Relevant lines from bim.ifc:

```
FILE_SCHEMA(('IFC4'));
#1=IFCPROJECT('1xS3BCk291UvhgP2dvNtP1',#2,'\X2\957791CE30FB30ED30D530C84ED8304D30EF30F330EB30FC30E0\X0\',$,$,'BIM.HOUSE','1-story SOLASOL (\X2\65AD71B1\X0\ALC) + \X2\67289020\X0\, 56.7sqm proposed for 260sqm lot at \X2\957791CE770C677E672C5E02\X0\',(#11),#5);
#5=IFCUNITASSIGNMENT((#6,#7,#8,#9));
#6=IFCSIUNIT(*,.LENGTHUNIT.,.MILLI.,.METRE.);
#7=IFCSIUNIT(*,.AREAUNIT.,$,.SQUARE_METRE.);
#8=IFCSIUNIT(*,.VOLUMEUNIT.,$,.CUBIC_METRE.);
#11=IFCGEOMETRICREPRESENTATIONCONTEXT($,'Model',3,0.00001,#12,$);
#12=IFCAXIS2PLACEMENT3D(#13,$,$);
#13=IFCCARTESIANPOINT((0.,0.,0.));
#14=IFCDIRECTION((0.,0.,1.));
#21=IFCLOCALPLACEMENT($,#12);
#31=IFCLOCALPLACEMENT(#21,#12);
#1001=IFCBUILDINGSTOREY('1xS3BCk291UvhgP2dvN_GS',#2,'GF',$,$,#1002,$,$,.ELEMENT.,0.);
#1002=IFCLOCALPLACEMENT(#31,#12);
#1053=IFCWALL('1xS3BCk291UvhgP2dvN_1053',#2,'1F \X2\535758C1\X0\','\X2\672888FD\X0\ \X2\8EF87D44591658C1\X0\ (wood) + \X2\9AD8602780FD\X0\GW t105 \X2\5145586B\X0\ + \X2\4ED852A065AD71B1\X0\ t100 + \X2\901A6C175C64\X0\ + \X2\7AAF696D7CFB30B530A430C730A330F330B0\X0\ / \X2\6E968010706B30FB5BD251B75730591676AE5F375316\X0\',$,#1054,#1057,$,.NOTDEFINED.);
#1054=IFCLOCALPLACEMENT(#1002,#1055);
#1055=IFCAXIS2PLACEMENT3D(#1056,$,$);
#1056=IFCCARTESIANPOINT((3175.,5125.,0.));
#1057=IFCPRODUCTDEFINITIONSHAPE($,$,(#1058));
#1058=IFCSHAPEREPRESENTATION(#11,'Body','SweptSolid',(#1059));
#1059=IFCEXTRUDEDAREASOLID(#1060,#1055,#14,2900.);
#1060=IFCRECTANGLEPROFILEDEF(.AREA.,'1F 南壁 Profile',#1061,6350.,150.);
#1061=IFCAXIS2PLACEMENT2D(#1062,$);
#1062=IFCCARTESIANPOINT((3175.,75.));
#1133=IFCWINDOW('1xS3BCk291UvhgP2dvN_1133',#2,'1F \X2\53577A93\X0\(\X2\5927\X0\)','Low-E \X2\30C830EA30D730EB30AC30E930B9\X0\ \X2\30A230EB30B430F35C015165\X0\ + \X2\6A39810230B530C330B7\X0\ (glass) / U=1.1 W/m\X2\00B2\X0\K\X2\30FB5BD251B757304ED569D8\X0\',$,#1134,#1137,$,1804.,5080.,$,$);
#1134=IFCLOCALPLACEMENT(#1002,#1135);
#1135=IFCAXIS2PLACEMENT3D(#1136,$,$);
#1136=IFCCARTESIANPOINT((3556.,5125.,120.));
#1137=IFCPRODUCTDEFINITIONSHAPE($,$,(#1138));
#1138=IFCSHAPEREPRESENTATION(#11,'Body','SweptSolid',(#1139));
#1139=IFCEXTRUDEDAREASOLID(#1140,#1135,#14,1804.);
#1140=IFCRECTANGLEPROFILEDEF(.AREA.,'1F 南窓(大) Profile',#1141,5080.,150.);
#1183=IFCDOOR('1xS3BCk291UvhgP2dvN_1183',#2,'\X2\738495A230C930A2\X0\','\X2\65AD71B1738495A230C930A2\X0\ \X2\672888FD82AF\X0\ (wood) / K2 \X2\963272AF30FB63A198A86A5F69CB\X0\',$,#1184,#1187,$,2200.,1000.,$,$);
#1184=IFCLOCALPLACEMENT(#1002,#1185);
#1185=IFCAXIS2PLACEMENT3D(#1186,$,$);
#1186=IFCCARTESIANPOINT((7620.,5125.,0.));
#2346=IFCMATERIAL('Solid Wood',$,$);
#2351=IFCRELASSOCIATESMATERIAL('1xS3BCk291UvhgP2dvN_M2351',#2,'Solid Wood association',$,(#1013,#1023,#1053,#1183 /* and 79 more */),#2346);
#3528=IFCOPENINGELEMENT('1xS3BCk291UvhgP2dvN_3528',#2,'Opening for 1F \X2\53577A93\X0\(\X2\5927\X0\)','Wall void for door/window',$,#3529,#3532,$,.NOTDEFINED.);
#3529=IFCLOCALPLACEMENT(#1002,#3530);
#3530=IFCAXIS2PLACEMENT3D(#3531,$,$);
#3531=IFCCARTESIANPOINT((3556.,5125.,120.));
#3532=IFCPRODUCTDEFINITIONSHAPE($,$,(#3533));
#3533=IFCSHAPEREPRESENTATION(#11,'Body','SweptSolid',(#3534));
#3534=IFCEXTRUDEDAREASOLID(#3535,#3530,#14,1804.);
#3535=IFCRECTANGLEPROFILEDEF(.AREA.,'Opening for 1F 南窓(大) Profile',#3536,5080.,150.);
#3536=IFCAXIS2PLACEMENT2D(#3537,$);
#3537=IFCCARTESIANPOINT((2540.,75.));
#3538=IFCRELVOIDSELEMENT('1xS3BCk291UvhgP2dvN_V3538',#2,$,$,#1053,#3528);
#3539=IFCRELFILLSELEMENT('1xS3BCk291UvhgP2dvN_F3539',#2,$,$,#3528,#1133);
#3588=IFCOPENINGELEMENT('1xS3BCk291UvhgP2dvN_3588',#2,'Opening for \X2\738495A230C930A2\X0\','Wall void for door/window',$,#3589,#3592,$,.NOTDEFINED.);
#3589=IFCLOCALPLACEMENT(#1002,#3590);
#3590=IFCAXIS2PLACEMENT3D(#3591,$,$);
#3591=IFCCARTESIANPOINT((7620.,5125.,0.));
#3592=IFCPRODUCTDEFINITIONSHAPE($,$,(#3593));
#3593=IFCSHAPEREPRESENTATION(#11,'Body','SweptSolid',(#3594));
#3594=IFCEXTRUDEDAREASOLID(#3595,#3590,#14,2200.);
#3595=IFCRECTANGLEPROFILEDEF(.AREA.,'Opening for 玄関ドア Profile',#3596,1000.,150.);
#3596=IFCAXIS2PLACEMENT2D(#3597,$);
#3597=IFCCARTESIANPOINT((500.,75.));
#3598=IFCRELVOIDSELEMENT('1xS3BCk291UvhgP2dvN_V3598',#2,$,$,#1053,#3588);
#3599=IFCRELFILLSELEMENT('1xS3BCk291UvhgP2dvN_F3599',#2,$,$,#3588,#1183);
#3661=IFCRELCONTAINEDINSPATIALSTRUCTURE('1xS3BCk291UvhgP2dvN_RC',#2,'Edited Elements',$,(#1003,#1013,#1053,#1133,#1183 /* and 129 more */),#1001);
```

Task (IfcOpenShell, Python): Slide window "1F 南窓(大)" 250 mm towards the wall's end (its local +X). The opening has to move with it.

```python
import ifcopenshell
import ifcopenshell.api.geometry
import ifcopenshell.util.placement

model = ifcopenshell.open("bim.ifc")

window = model.by_id(1133)
opening = window.FillsVoids[0].RelatingOpeningElement
wall = opening.VoidsElements[0].RelatingBuildingElement

wall_matrix = ifcopenshell.util.placement.get_local_placement(wall.ObjectPlacement)
shift = wall_matrix[:3, 0] * 250.0
before = ifcopenshell.util.placement.get_local_placement(window.ObjectPlacement)[:3, 3].copy()

# The window is not placed relative to its opening, so move both.
for product in (opening, window):
    matrix = ifcopenshell.util.placement.get_local_placement(product.ObjectPlacement)
    matrix[:3, 3] += shift
    ifcopenshell.api.geometry.edit_object_placement(model, product=product, matrix=matrix, is_si=False)

after = ifcopenshell.util.placement.get_local_placement(window.ObjectPlacement)[:3, 3]
print("window moved by", (after - before).round(3) + 0.0)

model.write("bim_edited.ifc")
```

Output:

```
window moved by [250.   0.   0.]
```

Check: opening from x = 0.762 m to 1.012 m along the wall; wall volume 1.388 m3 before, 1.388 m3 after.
